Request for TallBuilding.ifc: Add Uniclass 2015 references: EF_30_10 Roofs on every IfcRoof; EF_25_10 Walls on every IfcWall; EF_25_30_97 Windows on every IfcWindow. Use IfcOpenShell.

First a look at what the model holds.

```python
import ifcopenshell

model = ifcopenshell.open("TallBuilding.ifc")
print(model.schema)
print("classifications:", [c.Name for c in model.by_type("IfcClassification")])
for ifc_class in ("IfcDoor", "IfcRoof", "IfcStair", "IfcWall", "IfcWindow"):
    print(ifc_class, len(model.by_type(ifc_class)))
```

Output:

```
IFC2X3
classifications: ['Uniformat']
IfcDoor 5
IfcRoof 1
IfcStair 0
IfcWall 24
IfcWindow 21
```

```python
import ifcopenshell
import ifcopenshell.api.classification

model = ifcopenshell.open("TallBuilding.ifc")

# IFC2X3 requires Source and Edition and has no link from the project to the system.
system = model.create_entity("IfcClassification", Source="NBS", Edition="2015", Name="Uniclass 2015")

codes = {
    "IfcRoof": ("EF_30_10", "Roofs"),
    "IfcWall": ("EF_25_10", "Walls"),
    "IfcWindow": ("EF_25_30_97", "Windows"),
}
for ifc_class, (code, name) in codes.items():
    products = model.by_type(ifc_class)
    ifcopenshell.api.classification.add_reference(
        model, products=products, classification=system, identification=code, name=name
    )
    print(code, len(products))

model.write("TallBuilding_updated.ifc")
```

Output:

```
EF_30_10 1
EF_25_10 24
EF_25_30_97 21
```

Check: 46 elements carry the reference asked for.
